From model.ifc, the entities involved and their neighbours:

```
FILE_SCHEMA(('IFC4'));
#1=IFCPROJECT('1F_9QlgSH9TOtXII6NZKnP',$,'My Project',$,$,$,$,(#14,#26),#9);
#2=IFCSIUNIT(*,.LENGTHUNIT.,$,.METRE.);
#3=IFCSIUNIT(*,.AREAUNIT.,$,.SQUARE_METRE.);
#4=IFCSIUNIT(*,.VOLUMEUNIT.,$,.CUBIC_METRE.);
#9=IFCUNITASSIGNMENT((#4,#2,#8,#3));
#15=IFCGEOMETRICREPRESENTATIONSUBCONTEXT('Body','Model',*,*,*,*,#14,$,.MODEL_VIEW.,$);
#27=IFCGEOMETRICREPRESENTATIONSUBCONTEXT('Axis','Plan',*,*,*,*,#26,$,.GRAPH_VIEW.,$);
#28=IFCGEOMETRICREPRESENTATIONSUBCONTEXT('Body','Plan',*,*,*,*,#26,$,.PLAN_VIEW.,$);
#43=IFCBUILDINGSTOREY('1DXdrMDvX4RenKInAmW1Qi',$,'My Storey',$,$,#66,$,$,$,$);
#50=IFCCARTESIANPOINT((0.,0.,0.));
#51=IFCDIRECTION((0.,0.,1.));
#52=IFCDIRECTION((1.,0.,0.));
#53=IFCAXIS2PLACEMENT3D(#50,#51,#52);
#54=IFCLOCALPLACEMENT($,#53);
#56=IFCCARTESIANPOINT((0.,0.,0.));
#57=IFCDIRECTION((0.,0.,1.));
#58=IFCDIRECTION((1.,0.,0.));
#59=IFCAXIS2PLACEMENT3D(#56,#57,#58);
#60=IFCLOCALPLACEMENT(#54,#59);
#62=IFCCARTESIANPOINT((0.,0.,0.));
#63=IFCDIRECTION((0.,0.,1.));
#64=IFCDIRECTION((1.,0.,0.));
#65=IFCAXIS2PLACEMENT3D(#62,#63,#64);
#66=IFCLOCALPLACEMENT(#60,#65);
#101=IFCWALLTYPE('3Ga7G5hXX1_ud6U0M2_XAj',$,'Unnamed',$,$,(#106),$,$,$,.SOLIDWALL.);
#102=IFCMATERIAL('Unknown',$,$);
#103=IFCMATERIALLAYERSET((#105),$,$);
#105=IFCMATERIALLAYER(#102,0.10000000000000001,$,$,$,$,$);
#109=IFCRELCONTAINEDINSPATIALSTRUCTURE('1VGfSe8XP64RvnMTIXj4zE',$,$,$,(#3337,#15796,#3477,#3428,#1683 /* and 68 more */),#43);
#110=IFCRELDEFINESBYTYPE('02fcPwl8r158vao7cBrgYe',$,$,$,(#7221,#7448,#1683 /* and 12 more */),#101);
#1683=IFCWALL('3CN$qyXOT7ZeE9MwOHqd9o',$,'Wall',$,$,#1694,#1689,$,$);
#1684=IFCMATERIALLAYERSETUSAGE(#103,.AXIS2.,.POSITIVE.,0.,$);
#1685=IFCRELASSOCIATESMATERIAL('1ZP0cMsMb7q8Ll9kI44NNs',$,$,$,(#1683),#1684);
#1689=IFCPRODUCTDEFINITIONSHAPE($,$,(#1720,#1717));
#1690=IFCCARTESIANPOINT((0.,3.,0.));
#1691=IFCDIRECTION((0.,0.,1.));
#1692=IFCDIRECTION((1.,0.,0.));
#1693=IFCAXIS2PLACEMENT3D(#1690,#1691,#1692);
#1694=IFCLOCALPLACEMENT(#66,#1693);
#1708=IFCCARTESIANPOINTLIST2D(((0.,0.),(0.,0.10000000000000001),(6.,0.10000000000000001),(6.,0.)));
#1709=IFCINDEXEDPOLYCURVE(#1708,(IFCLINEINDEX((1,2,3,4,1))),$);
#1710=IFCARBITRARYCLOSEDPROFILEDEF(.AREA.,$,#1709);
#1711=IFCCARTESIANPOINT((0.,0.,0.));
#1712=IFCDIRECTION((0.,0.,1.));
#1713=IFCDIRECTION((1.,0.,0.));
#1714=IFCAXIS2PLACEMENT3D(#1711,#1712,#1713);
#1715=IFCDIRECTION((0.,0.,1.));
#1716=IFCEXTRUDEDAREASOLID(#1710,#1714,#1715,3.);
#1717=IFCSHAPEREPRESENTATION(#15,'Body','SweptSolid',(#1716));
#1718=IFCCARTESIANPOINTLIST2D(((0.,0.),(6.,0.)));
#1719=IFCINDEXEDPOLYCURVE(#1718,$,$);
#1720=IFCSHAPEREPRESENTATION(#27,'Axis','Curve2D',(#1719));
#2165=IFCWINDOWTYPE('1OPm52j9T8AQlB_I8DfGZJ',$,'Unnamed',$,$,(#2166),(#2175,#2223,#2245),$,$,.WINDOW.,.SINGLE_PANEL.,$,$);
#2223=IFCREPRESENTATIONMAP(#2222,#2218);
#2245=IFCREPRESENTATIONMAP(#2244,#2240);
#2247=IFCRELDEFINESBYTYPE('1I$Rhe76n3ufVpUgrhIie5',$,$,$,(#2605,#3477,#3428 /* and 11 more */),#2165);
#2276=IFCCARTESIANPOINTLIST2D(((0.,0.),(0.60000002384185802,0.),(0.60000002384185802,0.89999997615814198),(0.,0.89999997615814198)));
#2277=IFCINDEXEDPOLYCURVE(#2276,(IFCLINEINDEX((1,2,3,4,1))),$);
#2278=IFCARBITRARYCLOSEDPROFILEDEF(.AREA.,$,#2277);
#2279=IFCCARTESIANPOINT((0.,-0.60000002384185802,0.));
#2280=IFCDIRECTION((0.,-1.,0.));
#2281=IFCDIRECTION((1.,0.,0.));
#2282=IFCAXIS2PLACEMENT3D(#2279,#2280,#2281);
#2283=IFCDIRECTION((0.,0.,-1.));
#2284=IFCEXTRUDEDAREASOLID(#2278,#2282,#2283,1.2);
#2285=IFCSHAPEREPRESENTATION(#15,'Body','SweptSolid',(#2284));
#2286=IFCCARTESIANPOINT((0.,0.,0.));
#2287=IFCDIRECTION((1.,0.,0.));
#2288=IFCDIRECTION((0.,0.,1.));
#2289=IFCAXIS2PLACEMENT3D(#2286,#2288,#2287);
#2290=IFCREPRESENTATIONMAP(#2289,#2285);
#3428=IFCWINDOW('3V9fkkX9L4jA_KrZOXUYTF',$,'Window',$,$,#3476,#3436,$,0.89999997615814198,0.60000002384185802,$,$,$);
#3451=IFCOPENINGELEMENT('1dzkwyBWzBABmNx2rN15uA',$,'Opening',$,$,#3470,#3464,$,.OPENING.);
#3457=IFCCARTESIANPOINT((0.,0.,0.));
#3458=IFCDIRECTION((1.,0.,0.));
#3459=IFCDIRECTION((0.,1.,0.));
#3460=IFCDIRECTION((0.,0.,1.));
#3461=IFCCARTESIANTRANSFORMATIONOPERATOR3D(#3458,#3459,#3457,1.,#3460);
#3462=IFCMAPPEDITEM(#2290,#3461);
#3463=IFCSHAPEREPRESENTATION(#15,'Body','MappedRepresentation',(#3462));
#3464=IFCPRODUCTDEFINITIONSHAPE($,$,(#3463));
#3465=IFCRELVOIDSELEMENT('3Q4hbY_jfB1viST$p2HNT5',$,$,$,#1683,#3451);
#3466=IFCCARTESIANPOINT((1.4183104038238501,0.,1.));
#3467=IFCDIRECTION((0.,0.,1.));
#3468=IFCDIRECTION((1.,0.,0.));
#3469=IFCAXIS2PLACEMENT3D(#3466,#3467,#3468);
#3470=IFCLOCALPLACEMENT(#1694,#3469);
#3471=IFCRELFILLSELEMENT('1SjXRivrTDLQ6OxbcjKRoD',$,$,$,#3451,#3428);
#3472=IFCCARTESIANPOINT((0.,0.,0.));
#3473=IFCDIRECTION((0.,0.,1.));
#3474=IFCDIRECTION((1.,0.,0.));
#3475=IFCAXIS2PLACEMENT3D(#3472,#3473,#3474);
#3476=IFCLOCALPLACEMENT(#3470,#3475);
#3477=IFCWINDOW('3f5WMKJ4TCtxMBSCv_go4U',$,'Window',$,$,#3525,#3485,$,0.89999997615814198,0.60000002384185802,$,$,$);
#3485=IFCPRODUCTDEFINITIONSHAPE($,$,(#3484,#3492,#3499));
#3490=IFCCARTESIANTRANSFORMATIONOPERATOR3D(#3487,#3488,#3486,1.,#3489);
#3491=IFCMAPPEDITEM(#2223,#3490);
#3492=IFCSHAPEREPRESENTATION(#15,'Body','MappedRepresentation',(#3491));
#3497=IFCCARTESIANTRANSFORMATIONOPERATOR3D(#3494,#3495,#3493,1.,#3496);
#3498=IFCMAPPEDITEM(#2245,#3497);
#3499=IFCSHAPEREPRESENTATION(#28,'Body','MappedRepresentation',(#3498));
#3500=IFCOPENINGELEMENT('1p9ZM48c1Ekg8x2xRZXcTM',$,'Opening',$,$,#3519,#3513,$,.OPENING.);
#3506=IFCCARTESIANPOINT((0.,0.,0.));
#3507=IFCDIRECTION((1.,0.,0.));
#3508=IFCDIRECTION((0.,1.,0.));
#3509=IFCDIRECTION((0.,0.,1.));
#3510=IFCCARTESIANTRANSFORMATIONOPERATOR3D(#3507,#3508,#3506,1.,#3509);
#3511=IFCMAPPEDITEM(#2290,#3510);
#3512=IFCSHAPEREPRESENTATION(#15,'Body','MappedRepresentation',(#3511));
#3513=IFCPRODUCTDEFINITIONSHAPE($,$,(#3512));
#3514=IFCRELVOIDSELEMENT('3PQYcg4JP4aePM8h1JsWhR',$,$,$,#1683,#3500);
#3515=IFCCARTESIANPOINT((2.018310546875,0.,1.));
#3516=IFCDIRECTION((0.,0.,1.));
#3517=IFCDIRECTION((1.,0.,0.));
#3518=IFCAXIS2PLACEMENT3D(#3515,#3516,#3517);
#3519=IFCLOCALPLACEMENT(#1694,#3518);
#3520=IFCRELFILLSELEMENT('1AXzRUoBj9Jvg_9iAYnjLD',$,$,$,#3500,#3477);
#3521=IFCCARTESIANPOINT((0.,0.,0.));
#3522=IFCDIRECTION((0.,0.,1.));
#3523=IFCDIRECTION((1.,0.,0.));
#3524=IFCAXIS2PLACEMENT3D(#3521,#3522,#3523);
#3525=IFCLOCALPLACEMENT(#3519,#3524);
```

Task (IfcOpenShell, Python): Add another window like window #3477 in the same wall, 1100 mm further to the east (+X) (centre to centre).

```python
import ifcopenshell
import ifcopenshell.api.feature
import ifcopenshell.api.geometry
import ifcopenshell.api.root
import ifcopenshell.geom
import ifcopenshell.util.element
import ifcopenshell.util.placement
import ifcopenshell.util.shape
import ifcopenshell.util.unit

model = ifcopenshell.open("model.ifc")
unit_scale = ifcopenshell.util.unit.calculate_unit_scale(model)
settings = ifcopenshell.geom.settings()


def volume(element):
    """Net volume in cubic metres, openings subtracted."""
    shape = ifcopenshell.geom.create_shape(settings, element)
    return ifcopenshell.util.shape.get_volume(shape.geometry)


window = model.by_id(3477)
opening = window.FillsVoids[0].RelatingOpeningElement
wall = opening.VoidsElements[0].RelatingBuildingElement
before = volume(wall)
shift = ifcopenshell.util.placement.get_local_placement(wall.ObjectPlacement)[:3, 0] * 1.1 / unit_scale

# copy_class copies the void relationship, type, container and properties, but no geometry.
new_opening = ifcopenshell.api.root.copy_class(model, product=opening)
new_opening.Representation = ifcopenshell.util.element.copy_deep(
    model, opening.Representation, exclude=["IfcGeometricRepresentationContext", "IfcRepresentationMap"]
)
new_window = ifcopenshell.api.root.copy_class(model, product=window)
new_window.Representation = ifcopenshell.util.element.copy_deep(
    model, window.Representation, exclude=["IfcGeometricRepresentationContext", "IfcRepresentationMap"]
)
ifcopenshell.api.feature.add_filling(model, opening=new_opening, element=new_window)

for old, new in ((opening, new_opening), (window, new_window)):
    matrix = ifcopenshell.util.placement.get_local_placement(old.ObjectPlacement)
    matrix[:3, 3] += shift
    ifcopenshell.api.geometry.edit_object_placement(model, product=new, matrix=matrix, is_si=False)

after = volume(wall)

print(f"wall volume {before:.3f} -> {after:.3f} m3")

model.write("model_updated.ifc")
```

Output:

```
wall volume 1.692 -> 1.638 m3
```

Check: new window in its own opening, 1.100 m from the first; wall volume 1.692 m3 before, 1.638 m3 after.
